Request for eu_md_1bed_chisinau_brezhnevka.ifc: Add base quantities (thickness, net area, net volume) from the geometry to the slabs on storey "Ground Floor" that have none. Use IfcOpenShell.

First a look at what the model holds.

```python
import ifcopenshell
import ifcopenshell.util.element
import ifcopenshell.util.unit

model = ifcopenshell.open("eu_md_1bed_chisinau_brezhnevka.ifc")
print(model.schema)
for unit_type in ("LENGTHUNIT", "AREAUNIT", "VOLUMEUNIT"):
    print(unit_type, ifcopenshell.util.unit.calculate_unit_scale(model, unit_type))
storey = next(s for s in model.by_type("IfcBuildingStorey") if s.Name == "Ground Floor")
slabs = [e for e in ifcopenshell.util.element.get_decomposition(storey) if e.is_a("IfcSlab")]
for e in sorted(slabs, key=lambda e: e.id()):
    print(e.id(), e.is_a(), e.Name, list(ifcopenshell.util.element.get_psets(e, qtos_only=True)), sep=" | ")
```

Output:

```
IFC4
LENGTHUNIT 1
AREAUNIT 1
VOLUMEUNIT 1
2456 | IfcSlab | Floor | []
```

```python
import ifcopenshell
import ifcopenshell.api.pset
import ifcopenshell.geom
import ifcopenshell.util.element
import ifcopenshell.util.shape
import ifcopenshell.util.unit

model = ifcopenshell.open("eu_md_1bed_chisinau_brezhnevka.ifc")
unit_scale = ifcopenshell.util.unit.calculate_unit_scale(model)
area_scale = ifcopenshell.util.unit.calculate_unit_scale(model, "AREAUNIT")
volume_scale = ifcopenshell.util.unit.calculate_unit_scale(model, "VOLUMEUNIT")
settings = ifcopenshell.geom.settings()

storey = next(s for s in model.by_type("IfcBuildingStorey") if s.Name == "Ground Floor")
slabs = [e for e in ifcopenshell.util.element.get_decomposition(storey) if e.is_a("IfcSlab")]

for e in sorted(slabs, key=lambda e: e.id()):
    if ifcopenshell.util.element.get_psets(e, qtos_only=True, should_inherit=False):
        continue
    # Geometry comes back in metres, in the element's own axes.
    shape = ifcopenshell.geom.create_shape(settings, e)
    values = {
        "Width": ifcopenshell.util.shape.get_z(shape.geometry) / unit_scale,
        "NetArea": ifcopenshell.util.shape.get_footprint_area(shape.geometry) / area_scale,
        "NetVolume": ifcopenshell.util.shape.get_volume(shape.geometry) / volume_scale,
    }
    qto = ifcopenshell.api.pset.add_qto(model, product=e, name="Qto_SlabBaseQuantities")
    ifcopenshell.api.pset.edit_qto(model, qto=qto, properties=values)
    print(e.id(), {k: round(v, 3) for k, v in values.items()})

model.write("eu_md_1bed_chisinau_brezhnevka_v2.ifc")
```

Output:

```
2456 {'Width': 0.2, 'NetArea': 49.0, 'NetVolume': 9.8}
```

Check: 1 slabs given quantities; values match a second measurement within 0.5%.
